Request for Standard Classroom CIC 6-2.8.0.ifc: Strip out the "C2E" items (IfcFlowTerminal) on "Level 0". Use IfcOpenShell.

First a look at what the model holds.

```python
import ifcopenshell
import ifcopenshell.util.element

model = ifcopenshell.open("Standard Classroom CIC 6-2.8.0.ifc")
print(model.schema)
storey = next(s for s in model.by_type("IfcBuildingStorey") if s.Name == "Level 0")
terminals = [e for e in ifcopenshell.util.element.get_decomposition(storey) if e.is_a("IfcFlowTerminal")]
seen = {}
for e in terminals:
    element_type = ifcopenshell.util.element.get_type(e)
    name = element_type.Name if element_type not in (None, e) else None
    seen[name] = seen.get(name, 0) + 1
for name, count in sorted(seen.items(), key=str):
    print(count, "x", name)
```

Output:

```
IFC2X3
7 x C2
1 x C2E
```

```python
import ifcopenshell
import ifcopenshell.api.root
import ifcopenshell.util.element

model = ifcopenshell.open("Standard Classroom CIC 6-2.8.0.ifc")

storey = next(s for s in model.by_type("IfcBuildingStorey") if s.Name == "Level 0")
terminals = [e for e in ifcopenshell.util.element.get_decomposition(storey) if e.is_a("IfcFlowTerminal")]
targets = [e for e in terminals if (t := ifcopenshell.util.element.get_type(e)) not in (None, e) and t.Name == "C2E"]

for e in targets:
    ifcopenshell.api.root.remove_product(model, product=e)
print(len(targets), "removed")

model.write("Standard Classroom CIC 6-2.8.0-out.ifc")
```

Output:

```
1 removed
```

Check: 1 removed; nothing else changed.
